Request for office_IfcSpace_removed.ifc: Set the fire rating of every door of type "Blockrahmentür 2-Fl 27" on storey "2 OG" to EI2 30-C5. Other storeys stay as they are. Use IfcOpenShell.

First a look at what the model holds.

```python
import ifcopenshell
import ifcopenshell.util.element

model = ifcopenshell.open("office_IfcSpace_removed.ifc")
print(model.schema)
storey = next(s for s in model.by_type("IfcBuildingStorey") if s.Name == "2 OG")
doors = [e for e in ifcopenshell.util.element.get_decomposition(storey) if e.is_a("IfcDoor")]
seen = {}
for e in doors:
    element_type = ifcopenshell.util.element.get_type(e)
    key = (element_type.Name if element_type != e and element_type else None, ifcopenshell.util.element.get_pset(e, "Pset_DoorCommon", "FireRating"))
    seen[key] = seen.get(key, 0) + 1
for (name, value), count in sorted(seen.items(), key=str):
    print(count, "x", name, "|", value)
```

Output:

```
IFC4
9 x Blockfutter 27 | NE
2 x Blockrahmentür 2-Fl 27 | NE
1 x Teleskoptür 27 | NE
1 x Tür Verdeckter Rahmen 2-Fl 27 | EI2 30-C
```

```python
import ifcopenshell
import ifcopenshell.api.pset
import ifcopenshell.util.element

model = ifcopenshell.open("office_IfcSpace_removed.ifc")

storey = next(s for s in model.by_type("IfcBuildingStorey") if s.Name == "2 OG")
doors = [e for e in ifcopenshell.util.element.get_decomposition(storey) if e.is_a("IfcDoor")]

count = 0
for e in doors:
    element_type = ifcopenshell.util.element.get_type(e)
    if element_type in (None, e) or element_type.Name != "Blockrahmentür 2-Fl 27":
        continue
    # add_pset returns the element's existing set when there is one.
    pset = ifcopenshell.api.pset.add_pset(model, product=e, name="Pset_DoorCommon")
    ifcopenshell.api.pset.edit_pset(model, pset=pset, properties={"FireRating": "EI2 30-C5"})
    count += 1

print(count, "doors updated")

model.write("office_IfcSpace_removed_edited.ifc")
```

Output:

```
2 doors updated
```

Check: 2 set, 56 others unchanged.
